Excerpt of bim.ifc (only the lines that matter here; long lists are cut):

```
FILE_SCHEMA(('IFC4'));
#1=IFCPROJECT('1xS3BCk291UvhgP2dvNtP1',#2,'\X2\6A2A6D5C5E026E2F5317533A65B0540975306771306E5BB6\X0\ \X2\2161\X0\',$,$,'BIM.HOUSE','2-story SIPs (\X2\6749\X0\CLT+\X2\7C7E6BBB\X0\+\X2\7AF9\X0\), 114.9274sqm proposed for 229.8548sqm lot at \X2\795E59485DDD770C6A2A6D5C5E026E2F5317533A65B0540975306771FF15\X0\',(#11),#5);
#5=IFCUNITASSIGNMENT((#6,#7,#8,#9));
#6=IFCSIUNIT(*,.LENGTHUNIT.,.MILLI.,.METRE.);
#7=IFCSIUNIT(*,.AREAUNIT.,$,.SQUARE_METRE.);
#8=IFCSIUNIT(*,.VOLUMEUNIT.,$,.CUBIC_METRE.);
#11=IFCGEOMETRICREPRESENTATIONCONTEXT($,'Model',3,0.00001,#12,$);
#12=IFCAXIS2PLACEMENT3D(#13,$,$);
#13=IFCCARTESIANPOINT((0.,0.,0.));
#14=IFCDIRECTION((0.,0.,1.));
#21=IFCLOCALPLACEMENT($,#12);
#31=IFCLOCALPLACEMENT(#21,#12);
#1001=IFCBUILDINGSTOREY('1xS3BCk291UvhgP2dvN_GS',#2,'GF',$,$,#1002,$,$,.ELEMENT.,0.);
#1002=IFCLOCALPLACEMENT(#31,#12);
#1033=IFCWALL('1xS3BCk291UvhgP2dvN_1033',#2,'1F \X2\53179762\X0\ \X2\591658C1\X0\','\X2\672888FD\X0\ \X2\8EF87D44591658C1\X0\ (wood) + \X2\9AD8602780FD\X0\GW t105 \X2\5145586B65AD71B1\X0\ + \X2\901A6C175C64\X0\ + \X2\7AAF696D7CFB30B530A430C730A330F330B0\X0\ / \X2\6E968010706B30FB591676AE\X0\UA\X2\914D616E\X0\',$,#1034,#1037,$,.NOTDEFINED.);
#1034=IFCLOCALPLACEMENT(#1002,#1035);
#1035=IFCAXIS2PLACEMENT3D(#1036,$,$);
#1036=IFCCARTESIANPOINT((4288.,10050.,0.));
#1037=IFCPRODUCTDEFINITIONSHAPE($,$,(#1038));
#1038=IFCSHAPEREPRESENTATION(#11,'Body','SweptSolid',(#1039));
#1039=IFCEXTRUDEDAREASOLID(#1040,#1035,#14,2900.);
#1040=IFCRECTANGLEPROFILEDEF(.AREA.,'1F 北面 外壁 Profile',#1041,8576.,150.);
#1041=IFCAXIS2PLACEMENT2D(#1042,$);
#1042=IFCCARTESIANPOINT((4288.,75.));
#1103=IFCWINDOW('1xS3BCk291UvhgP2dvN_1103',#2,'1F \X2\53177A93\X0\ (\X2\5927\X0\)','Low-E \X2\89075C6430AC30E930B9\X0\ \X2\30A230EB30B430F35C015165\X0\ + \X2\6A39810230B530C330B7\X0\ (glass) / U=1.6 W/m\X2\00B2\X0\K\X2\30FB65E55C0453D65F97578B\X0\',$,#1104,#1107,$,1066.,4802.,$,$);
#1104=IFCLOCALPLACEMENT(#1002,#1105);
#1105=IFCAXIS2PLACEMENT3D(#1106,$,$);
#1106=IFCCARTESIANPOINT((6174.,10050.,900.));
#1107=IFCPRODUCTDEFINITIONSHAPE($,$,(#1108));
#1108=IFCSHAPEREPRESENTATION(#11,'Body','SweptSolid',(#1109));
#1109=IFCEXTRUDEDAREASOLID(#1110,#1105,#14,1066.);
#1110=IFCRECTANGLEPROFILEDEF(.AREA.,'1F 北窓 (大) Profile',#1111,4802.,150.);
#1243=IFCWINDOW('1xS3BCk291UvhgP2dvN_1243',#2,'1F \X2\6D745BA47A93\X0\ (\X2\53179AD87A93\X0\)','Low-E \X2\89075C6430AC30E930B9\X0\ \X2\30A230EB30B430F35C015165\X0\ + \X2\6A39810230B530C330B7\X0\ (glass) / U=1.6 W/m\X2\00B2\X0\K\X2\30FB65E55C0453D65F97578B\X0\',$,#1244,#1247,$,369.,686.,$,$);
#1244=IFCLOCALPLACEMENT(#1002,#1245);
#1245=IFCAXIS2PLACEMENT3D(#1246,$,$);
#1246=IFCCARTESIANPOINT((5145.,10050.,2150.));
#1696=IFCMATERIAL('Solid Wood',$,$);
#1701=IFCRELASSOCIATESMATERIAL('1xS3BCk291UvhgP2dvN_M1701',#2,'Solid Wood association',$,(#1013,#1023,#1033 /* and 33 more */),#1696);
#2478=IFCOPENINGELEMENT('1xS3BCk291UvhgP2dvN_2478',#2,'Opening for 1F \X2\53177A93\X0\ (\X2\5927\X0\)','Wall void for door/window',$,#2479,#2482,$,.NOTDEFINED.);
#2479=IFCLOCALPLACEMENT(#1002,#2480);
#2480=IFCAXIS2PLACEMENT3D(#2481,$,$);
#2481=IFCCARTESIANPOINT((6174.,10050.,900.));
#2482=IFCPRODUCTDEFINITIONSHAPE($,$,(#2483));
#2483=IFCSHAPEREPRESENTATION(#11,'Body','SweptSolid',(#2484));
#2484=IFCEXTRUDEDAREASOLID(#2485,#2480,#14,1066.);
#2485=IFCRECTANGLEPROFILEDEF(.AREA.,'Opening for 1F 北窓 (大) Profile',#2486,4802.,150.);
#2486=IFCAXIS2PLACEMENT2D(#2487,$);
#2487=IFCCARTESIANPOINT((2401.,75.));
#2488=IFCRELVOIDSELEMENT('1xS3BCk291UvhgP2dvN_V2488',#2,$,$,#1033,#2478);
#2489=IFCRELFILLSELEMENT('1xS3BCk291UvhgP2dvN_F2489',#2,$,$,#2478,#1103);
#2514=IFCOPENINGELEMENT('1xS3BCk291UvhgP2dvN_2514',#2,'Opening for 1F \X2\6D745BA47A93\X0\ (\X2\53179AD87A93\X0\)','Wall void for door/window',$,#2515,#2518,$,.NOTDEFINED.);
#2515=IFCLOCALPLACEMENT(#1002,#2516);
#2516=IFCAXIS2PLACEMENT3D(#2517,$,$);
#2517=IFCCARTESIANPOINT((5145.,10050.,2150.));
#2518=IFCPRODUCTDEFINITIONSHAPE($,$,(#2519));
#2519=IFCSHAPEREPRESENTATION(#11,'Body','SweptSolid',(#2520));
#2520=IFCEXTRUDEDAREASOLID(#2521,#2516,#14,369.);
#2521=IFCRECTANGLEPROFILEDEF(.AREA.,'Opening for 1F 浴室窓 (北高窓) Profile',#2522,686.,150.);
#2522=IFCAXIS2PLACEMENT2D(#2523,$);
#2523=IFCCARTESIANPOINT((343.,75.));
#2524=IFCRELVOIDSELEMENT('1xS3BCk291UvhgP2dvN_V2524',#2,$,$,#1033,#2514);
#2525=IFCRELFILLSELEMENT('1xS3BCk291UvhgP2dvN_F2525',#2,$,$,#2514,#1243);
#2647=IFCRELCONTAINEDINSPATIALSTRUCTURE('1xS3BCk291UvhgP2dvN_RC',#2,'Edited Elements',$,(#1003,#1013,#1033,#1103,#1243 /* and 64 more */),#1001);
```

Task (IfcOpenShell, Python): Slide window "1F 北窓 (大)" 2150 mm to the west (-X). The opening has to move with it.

```python
import ifcopenshell
import ifcopenshell.api.geometry
import ifcopenshell.util.placement
import ifcopenshell.util.unit

model = ifcopenshell.open("bim.ifc")
unit_scale = ifcopenshell.util.unit.calculate_unit_scale(model)

window = model.by_id(1103)
opening = window.FillsVoids[0].RelatingOpeningElement
wall = opening.VoidsElements[0].RelatingBuildingElement

wall_matrix = ifcopenshell.util.placement.get_local_placement(wall.ObjectPlacement)
shift = wall_matrix[:3, 0] * -2.15 / unit_scale
before = ifcopenshell.util.placement.get_local_placement(window.ObjectPlacement)[:3, 3].copy()

# The window is not placed relative to its opening, so move both.
for product in (opening, window):
    matrix = ifcopenshell.util.placement.get_local_placement(product.ObjectPlacement)
    matrix[:3, 3] += shift
    ifcopenshell.api.geometry.edit_object_placement(model, product=product, matrix=matrix, is_si=False)

after = ifcopenshell.util.placement.get_local_placement(window.ObjectPlacement)[:3, 3]
print("window moved by", (after - before).round(3) + 0.0)

model.write("bim-out.ifc")
```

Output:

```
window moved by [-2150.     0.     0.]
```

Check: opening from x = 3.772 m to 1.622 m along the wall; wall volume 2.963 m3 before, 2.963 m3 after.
